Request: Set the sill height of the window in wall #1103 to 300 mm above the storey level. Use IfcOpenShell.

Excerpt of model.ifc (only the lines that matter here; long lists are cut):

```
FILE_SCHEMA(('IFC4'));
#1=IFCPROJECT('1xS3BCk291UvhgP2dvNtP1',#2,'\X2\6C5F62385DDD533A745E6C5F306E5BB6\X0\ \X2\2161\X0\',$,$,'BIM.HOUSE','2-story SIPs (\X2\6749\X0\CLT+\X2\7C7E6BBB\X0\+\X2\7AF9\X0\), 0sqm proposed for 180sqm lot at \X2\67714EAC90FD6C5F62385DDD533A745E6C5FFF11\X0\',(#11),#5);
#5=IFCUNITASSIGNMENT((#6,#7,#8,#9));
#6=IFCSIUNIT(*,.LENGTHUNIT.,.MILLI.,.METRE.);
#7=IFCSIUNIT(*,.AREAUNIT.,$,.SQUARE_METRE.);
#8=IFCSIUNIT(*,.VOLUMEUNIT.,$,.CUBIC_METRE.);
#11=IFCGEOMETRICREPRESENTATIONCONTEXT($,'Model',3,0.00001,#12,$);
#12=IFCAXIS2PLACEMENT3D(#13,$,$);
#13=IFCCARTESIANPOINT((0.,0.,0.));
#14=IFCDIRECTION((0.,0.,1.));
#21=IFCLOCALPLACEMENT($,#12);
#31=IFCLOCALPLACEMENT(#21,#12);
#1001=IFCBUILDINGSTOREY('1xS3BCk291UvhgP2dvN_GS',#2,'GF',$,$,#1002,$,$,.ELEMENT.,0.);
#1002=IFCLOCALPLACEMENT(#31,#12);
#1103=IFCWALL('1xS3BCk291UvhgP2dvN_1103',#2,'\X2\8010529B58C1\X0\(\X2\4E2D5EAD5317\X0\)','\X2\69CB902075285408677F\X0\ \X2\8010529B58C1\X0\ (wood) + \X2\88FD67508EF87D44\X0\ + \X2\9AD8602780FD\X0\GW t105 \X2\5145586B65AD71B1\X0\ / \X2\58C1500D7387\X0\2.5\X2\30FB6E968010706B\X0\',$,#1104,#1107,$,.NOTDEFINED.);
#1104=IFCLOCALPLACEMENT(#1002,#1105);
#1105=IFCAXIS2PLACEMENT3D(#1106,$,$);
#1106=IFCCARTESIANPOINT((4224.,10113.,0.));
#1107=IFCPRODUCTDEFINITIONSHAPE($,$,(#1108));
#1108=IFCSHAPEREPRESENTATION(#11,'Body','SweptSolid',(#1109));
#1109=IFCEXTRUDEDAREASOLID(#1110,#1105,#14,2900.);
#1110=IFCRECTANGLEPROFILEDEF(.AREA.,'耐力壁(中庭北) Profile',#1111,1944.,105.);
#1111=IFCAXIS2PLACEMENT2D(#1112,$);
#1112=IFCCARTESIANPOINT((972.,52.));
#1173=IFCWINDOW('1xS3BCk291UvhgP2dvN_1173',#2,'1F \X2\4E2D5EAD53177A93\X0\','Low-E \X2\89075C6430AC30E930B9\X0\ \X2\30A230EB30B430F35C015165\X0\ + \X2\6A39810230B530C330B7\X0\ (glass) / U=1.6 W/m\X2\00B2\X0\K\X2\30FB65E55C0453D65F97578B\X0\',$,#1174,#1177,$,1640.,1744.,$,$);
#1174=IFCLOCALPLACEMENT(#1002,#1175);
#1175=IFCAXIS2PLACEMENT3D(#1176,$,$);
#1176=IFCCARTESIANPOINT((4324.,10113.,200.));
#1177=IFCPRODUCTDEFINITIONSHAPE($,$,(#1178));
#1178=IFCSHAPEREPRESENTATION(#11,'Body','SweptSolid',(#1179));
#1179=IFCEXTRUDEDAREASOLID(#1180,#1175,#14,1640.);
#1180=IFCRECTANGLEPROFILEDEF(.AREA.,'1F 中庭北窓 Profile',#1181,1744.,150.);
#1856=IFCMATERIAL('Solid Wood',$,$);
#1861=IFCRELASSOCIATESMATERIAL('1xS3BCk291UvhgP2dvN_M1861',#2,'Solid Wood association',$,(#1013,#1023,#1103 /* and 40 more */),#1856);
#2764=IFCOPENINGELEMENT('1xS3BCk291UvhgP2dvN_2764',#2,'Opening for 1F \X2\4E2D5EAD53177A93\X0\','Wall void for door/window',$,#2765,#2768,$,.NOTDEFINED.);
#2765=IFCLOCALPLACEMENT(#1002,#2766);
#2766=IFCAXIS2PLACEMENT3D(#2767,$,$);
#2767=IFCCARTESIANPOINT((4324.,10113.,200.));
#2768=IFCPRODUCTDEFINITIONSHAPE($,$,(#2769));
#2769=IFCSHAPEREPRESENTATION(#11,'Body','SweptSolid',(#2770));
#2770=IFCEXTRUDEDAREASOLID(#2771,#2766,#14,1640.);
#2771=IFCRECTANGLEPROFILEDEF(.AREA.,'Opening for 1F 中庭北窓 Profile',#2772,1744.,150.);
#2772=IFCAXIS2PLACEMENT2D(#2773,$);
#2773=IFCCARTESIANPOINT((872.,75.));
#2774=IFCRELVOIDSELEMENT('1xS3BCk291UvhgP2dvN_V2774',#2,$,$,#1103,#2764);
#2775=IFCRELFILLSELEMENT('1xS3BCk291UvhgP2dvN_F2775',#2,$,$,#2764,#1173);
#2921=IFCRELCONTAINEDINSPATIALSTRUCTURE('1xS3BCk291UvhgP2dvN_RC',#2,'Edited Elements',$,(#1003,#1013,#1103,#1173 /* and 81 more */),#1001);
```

```python
import numpy as np
import ifcopenshell
import ifcopenshell.api.geometry
import ifcopenshell.geom
import ifcopenshell.util.element
import ifcopenshell.util.placement
import ifcopenshell.util.shape
import ifcopenshell.util.unit

model = ifcopenshell.open("model.ifc")
unit_scale = ifcopenshell.util.unit.calculate_unit_scale(model)

window = model.by_guid("1xS3BCk291UvhgP2dvN_1173")
opening = window.FillsVoids[0].RelatingOpeningElement
storey = ifcopenshell.util.element.get_container(window, ifc_class="IfcBuildingStorey")
level = ifcopenshell.util.placement.get_local_placement(storey.ObjectPlacement)[2, 3]

# The opening's origin need not be at the sill, so measure its lowest point.
shape = ifcopenshell.geom.create_shape(ifcopenshell.geom.settings(), opening)
bottom = ifcopenshell.util.shape.get_shape_bottom_elevation(shape, shape.geometry) / unit_scale
dz = level + 0.3 / unit_scale - bottom

shift = np.array([0.0, 0.0, dz])
# The window is not placed relative to its opening, so move both.
for product in (opening, window):
    matrix = ifcopenshell.util.placement.get_local_placement(product.ObjectPlacement)
    matrix[:3, 3] += shift
    ifcopenshell.api.geometry.edit_object_placement(model, product=product, matrix=matrix, is_si=False)

print(f"moved by {dz * unit_scale:+.3f} m")

model.write("model_v2.ifc")
```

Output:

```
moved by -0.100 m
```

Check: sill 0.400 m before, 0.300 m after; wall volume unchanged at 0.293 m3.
